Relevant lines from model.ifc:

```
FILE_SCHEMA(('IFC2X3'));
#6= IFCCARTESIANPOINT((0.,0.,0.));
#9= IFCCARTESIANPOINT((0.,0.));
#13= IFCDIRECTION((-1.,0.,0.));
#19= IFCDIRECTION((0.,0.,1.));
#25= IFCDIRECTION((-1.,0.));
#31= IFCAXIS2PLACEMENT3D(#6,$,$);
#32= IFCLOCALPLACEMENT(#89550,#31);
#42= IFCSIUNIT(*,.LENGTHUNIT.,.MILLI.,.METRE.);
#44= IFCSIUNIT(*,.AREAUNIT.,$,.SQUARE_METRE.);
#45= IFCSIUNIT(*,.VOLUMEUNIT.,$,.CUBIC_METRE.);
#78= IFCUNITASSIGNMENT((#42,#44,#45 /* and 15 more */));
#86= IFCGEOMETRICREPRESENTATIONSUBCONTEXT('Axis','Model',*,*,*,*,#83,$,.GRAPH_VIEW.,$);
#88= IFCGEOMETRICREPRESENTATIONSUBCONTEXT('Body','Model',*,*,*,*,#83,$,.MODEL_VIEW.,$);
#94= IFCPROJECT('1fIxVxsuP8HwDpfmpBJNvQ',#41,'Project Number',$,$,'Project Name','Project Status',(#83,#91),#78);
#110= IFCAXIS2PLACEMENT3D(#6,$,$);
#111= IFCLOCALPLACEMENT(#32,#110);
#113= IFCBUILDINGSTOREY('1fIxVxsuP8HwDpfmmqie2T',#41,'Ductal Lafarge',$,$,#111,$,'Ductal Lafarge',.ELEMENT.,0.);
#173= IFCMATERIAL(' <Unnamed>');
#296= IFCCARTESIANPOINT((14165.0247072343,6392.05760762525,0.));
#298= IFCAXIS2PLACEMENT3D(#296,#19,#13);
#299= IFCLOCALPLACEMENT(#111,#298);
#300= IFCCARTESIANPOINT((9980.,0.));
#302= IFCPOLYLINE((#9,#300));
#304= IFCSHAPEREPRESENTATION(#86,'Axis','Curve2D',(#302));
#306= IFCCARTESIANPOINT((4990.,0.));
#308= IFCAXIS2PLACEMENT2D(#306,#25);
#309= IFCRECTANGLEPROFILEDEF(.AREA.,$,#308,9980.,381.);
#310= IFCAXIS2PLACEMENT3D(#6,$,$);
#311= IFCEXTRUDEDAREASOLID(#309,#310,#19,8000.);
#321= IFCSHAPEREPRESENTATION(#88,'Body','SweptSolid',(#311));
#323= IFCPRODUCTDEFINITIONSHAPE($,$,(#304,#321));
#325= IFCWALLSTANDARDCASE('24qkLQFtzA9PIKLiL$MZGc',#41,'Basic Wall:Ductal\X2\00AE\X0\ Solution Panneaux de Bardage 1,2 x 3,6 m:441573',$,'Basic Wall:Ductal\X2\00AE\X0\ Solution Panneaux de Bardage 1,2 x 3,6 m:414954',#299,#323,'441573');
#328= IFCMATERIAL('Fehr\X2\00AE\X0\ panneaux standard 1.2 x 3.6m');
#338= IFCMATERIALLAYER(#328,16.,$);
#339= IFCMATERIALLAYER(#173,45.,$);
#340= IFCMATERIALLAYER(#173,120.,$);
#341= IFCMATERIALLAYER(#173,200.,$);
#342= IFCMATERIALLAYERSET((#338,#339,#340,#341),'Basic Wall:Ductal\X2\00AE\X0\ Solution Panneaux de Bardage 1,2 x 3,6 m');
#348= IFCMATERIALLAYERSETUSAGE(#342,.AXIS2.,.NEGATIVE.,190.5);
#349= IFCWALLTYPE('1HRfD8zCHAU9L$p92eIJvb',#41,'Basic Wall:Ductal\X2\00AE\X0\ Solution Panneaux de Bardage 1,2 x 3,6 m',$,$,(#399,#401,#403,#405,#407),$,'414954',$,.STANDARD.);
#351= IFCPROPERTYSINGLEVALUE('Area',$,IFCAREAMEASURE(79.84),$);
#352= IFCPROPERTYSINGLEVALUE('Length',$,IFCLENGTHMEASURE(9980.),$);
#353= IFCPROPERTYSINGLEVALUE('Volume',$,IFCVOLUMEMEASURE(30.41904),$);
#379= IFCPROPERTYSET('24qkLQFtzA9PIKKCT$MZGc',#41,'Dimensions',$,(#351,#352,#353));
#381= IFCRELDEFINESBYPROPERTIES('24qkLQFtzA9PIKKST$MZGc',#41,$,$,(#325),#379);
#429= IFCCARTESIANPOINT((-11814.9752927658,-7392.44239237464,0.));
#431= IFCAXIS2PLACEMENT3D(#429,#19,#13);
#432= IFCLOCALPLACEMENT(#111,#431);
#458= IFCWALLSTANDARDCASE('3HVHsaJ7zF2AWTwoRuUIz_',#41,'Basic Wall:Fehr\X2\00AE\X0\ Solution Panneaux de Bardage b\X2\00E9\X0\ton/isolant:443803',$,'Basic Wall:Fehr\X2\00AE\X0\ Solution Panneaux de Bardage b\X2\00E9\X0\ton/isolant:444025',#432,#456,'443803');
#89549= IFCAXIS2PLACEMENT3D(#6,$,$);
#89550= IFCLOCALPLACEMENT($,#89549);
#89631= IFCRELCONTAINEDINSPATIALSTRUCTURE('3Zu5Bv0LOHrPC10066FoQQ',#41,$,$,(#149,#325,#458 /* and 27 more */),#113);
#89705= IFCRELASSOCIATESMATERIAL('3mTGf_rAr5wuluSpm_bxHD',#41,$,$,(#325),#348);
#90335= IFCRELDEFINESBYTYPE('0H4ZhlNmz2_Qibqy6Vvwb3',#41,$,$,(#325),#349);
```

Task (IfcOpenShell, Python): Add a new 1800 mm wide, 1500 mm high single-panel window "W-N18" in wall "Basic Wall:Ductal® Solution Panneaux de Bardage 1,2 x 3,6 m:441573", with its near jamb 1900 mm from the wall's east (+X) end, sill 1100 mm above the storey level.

```python
import numpy as np
import ifcopenshell
import ifcopenshell.api.feature
import ifcopenshell.api.geometry
import ifcopenshell.api.pset
import ifcopenshell.api.root
import ifcopenshell.api.spatial
import ifcopenshell.api.type
import ifcopenshell.geom
import ifcopenshell.util.element
import ifcopenshell.util.placement
import ifcopenshell.util.representation
import ifcopenshell.util.shape
import ifcopenshell.util.unit

model = ifcopenshell.open("model.ifc")
unit_scale = ifcopenshell.util.unit.calculate_unit_scale(model)
area_scale = ifcopenshell.util.unit.calculate_unit_scale(model, "AREAUNIT")
volume_scale = ifcopenshell.util.unit.calculate_unit_scale(model, "VOLUMEUNIT")
settings = ifcopenshell.geom.settings()


def volume(element):
    """Net volume in cubic metres, openings subtracted."""
    shape = ifcopenshell.geom.create_shape(settings, element)
    return ifcopenshell.util.shape.get_volume(shape.geometry)


wall = model.by_guid("24qkLQFtzA9PIKLiL$MZGc")
storey = ifcopenshell.util.element.get_container(wall, ifc_class="IfcBuildingStorey")
context = ifcopenshell.util.representation.get_context(model, "Model", "Body", "MODEL_VIEW")
before = volume(wall)

width, height, from_end, sill = 1.8, 1.5, 1.9, 1.1  # metres

# The wall runs along its own X axis, and the end named is its -X end.
wall_shape = ifcopenshell.geom.create_shape(settings, wall)
x, y, z = ifcopenshell.util.shape.get_vertices(wall_shape.geometry).T
start = x.min() + from_end
face, thickness = float(y.min()), float(y.max() - y.min())
wall_matrix = ifcopenshell.util.placement.get_local_placement(wall.ObjectPlacement)
level = ifcopenshell.util.placement.get_local_placement(storey.ObjectPlacement)[2, 3]


def in_wall(x, y):
    """Placement at x, y metres in the wall's axes, at sill height."""
    matrix = wall_matrix.copy()
    matrix[:, 3] = wall_matrix @ np.array([x / unit_scale, y / unit_scale, 0.0, 1.0])
    matrix[2, 3] = level + sill / unit_scale
    return matrix


# Opening: a box that overshoots both wall faces by 50 mm.
opening = ifcopenshell.api.root.create_entity(model, ifc_class="IfcOpeningElement")
box = ifcopenshell.api.geometry.add_wall_representation(
    model, context=context, length=width, height=height, thickness=thickness + 0.1
)
ifcopenshell.api.geometry.assign_representation(model, product=opening, representation=box)
ifcopenshell.api.geometry.edit_object_placement(model, product=opening, matrix=in_wall(start, face - 0.05), is_si=False)
ifcopenshell.api.feature.add_feature(model, feature=opening, element=wall)

window = ifcopenshell.api.root.create_entity(model, ifc_class="IfcWindow", name="W-N18")
window.OverallWidth, window.OverallHeight = width / unit_scale, height / unit_scale
body = ifcopenshell.api.geometry.add_window_representation(
    model,
    context=context,
    overall_width=window.OverallWidth,
    overall_height=window.OverallHeight,
    partition_type="SINGLE_PANEL",
)
ifcopenshell.api.geometry.assign_representation(model, product=window, representation=body)
ifcopenshell.api.spatial.assign_container(model, products=[window], relating_structure=storey)
fills = ifcopenshell.api.feature.add_filling(model, opening=opening, element=window)
fills.OwnerHistory = window.OwnerHistory  # required in IFC2X3

# IFC2X3 keeps the operation on the window style.
style = ifcopenshell.api.root.create_entity(model, ifc_class="IfcWindowStyle", name="W-N18")
style.OperationType, style.ConstructionType = "SINGLE_PANEL", "NOTDEFINED"
style.ParameterTakesPrecedence = style.Sizeable = False
ifcopenshell.api.type.assign_type(model, related_objects=[window], relating_type=style)

# Centre the window in the wall's thickness.
ifcopenshell.api.geometry.edit_object_placement(model, product=window, matrix=in_wall(start, face), is_si=False)
window_shape = ifcopenshell.geom.create_shape(settings, window)
depth = ifcopenshell.util.shape.get_vertices(window_shape.geometry)[:, 1]
offset = face + thickness / 2 - (depth.min() + depth.max()) / 2
ifcopenshell.api.geometry.edit_object_placement(model, product=window, matrix=in_wall(start, offset), is_si=False)

after = volume(wall)

# Update the wall's stored quantities.
pset = model.by_id(ifcopenshell.util.element.get_pset(wall, "Dimensions", should_inherit=False)["id"])
ifcopenshell.api.pset.edit_pset(model, pset=pset, properties={
    "Area": model.create_entity("IfcAreaMeasure", after / thickness / area_scale),
    "Volume": model.create_entity("IfcVolumeMeasure", after / volume_scale),
})

print(f"wall volume {before:.3f} -> {after:.3f} m3")

model.write("model_edited.ifc")
```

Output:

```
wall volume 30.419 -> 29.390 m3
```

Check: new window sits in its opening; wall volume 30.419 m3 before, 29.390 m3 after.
